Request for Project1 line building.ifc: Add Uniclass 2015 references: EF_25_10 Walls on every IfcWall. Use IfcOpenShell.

First a look at what the model holds.

```python
import ifcopenshell

model = ifcopenshell.open("Project1 line building.ifc")
print(model.schema)
print("classifications:", [c.Name for c in model.by_type("IfcClassification")])
for ifc_class in ("IfcDoor", "IfcRoof", "IfcStair", "IfcWall", "IfcWindow"):
    print(ifc_class, len(model.by_type(ifc_class)))
```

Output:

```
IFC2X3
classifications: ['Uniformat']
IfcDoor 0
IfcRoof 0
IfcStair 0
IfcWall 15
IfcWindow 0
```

```python
import ifcopenshell
import ifcopenshell.api.classification

model = ifcopenshell.open("Project1 line building.ifc")

# IFC2X3 requires Source and Edition and has no link from the project to the system.
system = model.create_entity("IfcClassification", Source="NBS", Edition="2015", Name="Uniclass 2015")

codes = {
    "IfcWall": ("EF_25_10", "Walls"),
}
for ifc_class, (code, name) in codes.items():
    products = model.by_type(ifc_class)
    ifcopenshell.api.classification.add_reference(
        model, products=products, classification=system, identification=code, name=name
    )
    print(code, len(products))

model.write("Project1 line building_rev.ifc")
```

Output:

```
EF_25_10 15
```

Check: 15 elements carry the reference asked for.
